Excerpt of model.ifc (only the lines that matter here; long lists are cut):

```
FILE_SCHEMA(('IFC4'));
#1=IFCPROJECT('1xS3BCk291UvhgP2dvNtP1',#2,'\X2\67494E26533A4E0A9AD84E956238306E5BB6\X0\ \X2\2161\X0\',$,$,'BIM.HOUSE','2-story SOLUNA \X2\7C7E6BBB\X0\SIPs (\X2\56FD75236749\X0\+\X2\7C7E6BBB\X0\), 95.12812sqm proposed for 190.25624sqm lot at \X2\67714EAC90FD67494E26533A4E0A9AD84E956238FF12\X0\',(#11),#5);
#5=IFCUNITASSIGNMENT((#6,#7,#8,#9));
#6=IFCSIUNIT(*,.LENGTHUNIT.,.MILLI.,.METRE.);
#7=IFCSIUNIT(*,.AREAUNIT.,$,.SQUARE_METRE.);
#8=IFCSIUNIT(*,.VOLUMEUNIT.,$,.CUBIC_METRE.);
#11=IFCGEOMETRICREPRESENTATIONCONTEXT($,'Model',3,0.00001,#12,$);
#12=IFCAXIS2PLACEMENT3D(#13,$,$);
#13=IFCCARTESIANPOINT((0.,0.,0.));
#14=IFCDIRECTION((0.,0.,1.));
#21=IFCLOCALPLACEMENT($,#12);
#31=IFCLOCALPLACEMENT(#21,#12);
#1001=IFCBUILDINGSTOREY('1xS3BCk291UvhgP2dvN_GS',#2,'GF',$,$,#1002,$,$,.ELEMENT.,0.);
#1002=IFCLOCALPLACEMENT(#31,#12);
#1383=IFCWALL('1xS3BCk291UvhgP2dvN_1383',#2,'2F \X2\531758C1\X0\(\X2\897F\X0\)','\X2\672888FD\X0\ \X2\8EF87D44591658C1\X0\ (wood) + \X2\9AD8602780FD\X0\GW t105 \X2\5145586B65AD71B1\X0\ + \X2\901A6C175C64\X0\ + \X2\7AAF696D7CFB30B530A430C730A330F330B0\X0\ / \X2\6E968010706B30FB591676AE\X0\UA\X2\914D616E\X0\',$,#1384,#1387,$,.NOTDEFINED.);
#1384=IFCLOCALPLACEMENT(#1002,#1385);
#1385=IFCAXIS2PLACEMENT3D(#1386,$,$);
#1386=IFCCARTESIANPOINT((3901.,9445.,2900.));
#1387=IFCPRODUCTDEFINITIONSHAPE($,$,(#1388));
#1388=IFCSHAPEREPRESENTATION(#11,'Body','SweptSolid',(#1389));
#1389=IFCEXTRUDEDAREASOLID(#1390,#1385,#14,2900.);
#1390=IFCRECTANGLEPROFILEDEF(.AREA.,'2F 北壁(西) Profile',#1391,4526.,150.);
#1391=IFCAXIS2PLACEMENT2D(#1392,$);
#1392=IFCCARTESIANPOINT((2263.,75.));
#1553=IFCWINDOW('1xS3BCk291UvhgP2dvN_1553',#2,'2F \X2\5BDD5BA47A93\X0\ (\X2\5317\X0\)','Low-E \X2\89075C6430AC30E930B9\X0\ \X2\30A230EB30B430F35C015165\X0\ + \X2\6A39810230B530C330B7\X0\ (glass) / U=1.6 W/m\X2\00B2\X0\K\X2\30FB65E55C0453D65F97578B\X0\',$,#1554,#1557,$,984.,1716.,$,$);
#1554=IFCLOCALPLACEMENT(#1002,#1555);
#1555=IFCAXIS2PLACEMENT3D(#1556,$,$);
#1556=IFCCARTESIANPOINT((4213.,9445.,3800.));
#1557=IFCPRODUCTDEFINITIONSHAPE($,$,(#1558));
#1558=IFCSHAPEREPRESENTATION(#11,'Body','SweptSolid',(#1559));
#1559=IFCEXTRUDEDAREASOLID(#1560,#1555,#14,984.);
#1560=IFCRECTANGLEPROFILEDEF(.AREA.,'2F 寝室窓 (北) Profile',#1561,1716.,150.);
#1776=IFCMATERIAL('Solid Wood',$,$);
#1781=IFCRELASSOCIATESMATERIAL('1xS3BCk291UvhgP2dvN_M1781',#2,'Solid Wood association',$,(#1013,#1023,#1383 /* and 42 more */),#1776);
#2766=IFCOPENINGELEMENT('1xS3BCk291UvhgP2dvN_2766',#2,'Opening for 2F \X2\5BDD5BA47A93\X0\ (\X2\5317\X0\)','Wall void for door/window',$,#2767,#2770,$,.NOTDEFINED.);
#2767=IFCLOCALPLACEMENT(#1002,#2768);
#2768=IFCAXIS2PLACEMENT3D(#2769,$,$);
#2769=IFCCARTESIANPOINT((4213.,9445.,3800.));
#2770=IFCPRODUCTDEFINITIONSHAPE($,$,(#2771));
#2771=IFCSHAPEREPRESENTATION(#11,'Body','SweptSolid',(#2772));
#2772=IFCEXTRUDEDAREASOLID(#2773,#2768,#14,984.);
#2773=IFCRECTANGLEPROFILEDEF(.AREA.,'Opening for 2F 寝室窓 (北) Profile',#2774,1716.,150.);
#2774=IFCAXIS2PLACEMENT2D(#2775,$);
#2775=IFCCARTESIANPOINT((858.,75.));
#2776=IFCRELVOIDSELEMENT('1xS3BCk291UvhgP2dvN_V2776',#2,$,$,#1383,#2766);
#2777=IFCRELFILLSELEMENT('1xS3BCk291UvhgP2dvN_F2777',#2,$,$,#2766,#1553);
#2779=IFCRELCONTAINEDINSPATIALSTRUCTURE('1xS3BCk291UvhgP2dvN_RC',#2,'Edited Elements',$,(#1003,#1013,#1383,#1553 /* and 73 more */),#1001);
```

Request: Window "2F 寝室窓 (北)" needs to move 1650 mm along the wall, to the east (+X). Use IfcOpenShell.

```python
import ifcopenshell
import ifcopenshell.api.geometry
import ifcopenshell.util.placement
import ifcopenshell.util.unit

model = ifcopenshell.open("model.ifc")
unit_scale = ifcopenshell.util.unit.calculate_unit_scale(model)

window = model.by_guid("1xS3BCk291UvhgP2dvN_1553")
opening = window.FillsVoids[0].RelatingOpeningElement
wall = opening.VoidsElements[0].RelatingBuildingElement

wall_matrix = ifcopenshell.util.placement.get_local_placement(wall.ObjectPlacement)
shift = wall_matrix[:3, 0] * 1.65 / unit_scale
before = ifcopenshell.util.placement.get_local_placement(window.ObjectPlacement)[:3, 3].copy()

# The window is not placed relative to its opening, so move both.
for product in (opening, window):
    matrix = ifcopenshell.util.placement.get_local_placement(product.ObjectPlacement)
    matrix[:3, 3] += shift
    ifcopenshell.api.geometry.edit_object_placement(model, product=product, matrix=matrix, is_si=False)

after = ifcopenshell.util.placement.get_local_placement(window.ObjectPlacement)[:3, 3]
print("window moved by", (after - before).round(3) + 0.0)

model.write("model-out.ifc")
```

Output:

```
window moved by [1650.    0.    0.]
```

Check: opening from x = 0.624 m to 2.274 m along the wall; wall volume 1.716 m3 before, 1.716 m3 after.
